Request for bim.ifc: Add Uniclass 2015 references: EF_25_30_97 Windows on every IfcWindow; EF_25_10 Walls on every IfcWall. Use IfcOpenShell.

First a look at what the model holds.

```python
import ifcopenshell

model = ifcopenshell.open("bim.ifc")
print(model.schema)
print("classifications:", [c.Name for c in model.by_type("IfcClassification")])
for ifc_class in ("IfcDoor", "IfcRoof", "IfcStair", "IfcWall", "IfcWindow"):
    print(ifc_class, len(model.by_type(ifc_class)))
```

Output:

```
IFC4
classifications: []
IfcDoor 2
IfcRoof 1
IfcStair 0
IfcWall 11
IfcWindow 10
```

```python
import ifcopenshell
import ifcopenshell.api.classification

model = ifcopenshell.open("bim.ifc")

system = ifcopenshell.api.classification.add_classification(model, classification="Uniclass 2015")

codes = {
    "IfcWindow": ("EF_25_30_97", "Windows"),
    "IfcWall": ("EF_25_10", "Walls"),
}
for ifc_class, (code, name) in codes.items():
    products = model.by_type(ifc_class)
    ifcopenshell.api.classification.add_reference(
        model, products=products, classification=system, identification=code, name=name
    )
    print(code, len(products))

model.write("bim-out.ifc")
```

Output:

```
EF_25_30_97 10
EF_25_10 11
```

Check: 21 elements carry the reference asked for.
